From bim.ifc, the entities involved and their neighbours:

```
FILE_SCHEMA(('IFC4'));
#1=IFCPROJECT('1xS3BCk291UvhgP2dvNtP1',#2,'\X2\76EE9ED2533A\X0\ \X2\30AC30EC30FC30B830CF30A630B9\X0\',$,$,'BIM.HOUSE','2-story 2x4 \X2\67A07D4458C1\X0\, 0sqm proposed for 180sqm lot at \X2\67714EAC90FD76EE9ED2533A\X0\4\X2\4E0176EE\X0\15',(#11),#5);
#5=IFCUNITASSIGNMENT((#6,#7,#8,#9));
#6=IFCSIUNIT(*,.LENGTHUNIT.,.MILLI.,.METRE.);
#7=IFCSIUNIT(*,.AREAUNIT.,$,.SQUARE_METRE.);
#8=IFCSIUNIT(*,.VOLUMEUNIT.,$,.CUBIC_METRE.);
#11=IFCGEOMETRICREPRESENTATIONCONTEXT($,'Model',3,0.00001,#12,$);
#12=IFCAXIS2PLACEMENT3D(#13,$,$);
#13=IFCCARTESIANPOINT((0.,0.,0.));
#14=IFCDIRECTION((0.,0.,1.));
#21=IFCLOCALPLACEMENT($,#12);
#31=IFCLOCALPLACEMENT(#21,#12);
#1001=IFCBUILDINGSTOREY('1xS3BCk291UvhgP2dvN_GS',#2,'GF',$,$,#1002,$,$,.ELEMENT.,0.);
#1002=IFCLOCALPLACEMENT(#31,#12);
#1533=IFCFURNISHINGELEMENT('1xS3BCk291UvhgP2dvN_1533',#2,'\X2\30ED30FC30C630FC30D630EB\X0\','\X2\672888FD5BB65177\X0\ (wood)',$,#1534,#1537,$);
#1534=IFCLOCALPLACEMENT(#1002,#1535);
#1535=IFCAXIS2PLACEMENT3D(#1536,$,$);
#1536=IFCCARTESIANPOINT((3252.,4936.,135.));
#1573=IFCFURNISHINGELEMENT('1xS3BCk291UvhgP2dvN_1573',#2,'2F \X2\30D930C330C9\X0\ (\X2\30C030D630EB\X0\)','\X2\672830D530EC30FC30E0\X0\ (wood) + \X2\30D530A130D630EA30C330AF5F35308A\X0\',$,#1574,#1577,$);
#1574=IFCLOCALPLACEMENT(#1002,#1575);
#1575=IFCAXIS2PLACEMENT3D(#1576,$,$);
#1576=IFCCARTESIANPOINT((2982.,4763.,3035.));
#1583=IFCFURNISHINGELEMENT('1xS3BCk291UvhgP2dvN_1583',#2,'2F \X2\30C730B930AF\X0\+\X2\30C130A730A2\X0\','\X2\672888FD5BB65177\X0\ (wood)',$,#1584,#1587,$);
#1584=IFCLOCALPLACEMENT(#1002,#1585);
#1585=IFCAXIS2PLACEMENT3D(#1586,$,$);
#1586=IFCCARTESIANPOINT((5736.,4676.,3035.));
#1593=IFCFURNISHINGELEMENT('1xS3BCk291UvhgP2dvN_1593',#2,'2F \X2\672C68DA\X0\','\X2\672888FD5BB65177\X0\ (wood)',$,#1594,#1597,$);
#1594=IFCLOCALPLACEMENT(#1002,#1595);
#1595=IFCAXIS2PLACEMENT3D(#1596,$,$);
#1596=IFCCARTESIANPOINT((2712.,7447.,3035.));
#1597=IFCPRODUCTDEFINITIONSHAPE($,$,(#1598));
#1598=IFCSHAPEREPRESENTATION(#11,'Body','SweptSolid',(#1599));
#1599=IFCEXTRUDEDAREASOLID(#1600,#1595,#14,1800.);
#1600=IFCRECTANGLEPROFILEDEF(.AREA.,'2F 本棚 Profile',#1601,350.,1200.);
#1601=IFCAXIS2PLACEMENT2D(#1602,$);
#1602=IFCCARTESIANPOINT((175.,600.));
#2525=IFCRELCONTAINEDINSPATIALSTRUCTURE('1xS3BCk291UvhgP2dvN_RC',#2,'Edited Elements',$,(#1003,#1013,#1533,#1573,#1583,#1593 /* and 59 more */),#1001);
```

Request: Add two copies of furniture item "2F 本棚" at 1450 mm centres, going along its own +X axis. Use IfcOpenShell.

```python
import ifcopenshell
import ifcopenshell.api.geometry
import ifcopenshell.api.root
import ifcopenshell.util.element
import ifcopenshell.util.placement
import ifcopenshell.util.unit

model = ifcopenshell.open("bim.ifc")
unit_scale = ifcopenshell.util.unit.calculate_unit_scale(model)


def reuse_history(source, copy):
    """copy_class also copies each property set's owner history, people and application; keep the originals."""
    for rel in copy.IsDefinedBy:
        if rel.is_a("IfcRelDefinesByProperties") and (history := rel.RelatingPropertyDefinition.OwnerHistory):
            rel.RelatingPropertyDefinition.OwnerHistory = source.OwnerHistory
            ifcopenshell.util.element.remove_deep2(model, history)


source = model.by_id(1593)
base = ifcopenshell.util.placement.get_local_placement(source.ObjectPlacement)
step = base[:3, 0] * 1.45 / unit_scale

for i in range(1, 3):
    copy = ifcopenshell.api.root.copy_class(model, product=source)
    copy.Representation = ifcopenshell.util.element.copy_deep(
        model, source.Representation, exclude=["IfcGeometricRepresentationContext", "IfcRepresentationMap"]
    )
    reuse_history(source, copy)
    matrix = base.copy()
    matrix[:3, 3] += i * step
    print("added at", matrix[:3, 3].round(3) + 0.0)
    ifcopenshell.api.geometry.edit_object_placement(model, product=copy, matrix=matrix, is_si=False)

model.write("bim_updated.ifc")
```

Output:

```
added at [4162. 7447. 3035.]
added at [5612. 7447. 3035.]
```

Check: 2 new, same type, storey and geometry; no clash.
